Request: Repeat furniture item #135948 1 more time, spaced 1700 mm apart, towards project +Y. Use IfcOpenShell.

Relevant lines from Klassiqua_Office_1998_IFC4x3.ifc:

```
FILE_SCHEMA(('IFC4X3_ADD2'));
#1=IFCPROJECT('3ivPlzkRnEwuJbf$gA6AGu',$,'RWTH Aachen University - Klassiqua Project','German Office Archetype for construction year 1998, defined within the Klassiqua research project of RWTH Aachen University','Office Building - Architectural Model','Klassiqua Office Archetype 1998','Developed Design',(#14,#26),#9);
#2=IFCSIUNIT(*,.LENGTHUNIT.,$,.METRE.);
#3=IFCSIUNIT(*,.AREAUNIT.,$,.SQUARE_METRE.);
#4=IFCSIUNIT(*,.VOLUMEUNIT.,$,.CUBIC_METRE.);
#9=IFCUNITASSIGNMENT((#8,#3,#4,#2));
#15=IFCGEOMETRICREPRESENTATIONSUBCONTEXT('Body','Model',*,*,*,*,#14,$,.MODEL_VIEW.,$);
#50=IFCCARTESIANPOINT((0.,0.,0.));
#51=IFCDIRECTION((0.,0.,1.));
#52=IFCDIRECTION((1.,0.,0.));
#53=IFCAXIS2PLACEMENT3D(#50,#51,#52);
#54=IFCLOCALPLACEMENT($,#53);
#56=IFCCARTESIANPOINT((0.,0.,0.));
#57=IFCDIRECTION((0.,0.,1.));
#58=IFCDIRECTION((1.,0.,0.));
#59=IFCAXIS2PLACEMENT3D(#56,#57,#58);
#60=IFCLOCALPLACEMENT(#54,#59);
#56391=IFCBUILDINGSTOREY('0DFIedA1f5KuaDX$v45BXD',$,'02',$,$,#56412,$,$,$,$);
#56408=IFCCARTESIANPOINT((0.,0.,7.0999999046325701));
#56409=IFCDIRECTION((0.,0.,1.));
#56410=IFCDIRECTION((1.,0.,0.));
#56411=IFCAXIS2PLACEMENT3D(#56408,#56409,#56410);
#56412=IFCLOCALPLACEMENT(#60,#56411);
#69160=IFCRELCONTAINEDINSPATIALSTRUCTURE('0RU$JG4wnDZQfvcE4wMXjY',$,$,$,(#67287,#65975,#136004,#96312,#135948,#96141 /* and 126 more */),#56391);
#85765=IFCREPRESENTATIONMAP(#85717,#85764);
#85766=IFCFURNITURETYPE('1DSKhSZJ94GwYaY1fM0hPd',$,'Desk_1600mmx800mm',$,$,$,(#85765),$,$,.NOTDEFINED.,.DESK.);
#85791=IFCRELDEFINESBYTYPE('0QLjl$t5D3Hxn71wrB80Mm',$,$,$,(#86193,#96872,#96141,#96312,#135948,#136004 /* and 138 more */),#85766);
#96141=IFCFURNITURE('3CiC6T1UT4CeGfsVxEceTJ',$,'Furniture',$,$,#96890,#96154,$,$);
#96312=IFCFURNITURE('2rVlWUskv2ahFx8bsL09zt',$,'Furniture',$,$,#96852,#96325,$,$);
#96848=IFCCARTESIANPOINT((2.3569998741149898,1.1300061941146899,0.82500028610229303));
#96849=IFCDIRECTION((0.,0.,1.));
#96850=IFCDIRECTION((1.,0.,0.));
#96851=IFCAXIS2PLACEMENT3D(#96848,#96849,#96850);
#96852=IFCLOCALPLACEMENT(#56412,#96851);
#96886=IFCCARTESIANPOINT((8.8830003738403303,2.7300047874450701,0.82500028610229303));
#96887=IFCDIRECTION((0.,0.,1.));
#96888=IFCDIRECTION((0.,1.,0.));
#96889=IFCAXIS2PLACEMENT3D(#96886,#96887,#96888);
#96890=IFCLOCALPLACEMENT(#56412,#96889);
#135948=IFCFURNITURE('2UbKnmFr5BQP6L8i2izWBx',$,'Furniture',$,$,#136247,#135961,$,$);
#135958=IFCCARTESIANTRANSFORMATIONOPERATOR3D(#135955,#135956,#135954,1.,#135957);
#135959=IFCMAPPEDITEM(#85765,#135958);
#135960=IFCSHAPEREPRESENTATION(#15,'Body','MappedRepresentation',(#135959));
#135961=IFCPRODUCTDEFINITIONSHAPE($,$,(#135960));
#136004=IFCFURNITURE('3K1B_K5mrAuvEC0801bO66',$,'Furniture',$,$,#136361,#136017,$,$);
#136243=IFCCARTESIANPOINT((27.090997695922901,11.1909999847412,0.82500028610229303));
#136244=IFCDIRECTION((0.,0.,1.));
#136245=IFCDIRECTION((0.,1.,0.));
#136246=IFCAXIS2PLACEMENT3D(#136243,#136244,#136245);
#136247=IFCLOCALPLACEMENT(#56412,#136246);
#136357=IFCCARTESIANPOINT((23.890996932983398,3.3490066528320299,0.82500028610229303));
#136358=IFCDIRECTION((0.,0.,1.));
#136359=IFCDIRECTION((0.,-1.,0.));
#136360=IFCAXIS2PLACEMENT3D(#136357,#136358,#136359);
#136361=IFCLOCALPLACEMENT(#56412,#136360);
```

```python
import numpy as np
import ifcopenshell
import ifcopenshell.api.geometry
import ifcopenshell.api.root
import ifcopenshell.util.element
import ifcopenshell.util.placement

model = ifcopenshell.open("Klassiqua_Office_1998_IFC4x3.ifc")

source = model.by_guid("2UbKnmFr5BQP6L8i2izWBx")
base = ifcopenshell.util.placement.get_local_placement(source.ObjectPlacement)
step = np.array([0.0, 1.0, 0.0]) * 1.7

for i in range(1, 2):
    copy = ifcopenshell.api.root.copy_class(model, product=source)
    copy.Representation = ifcopenshell.util.element.copy_deep(
        model, source.Representation, exclude=["IfcGeometricRepresentationContext", "IfcRepresentationMap"]
    )
    matrix = base.copy()
    matrix[:3, 3] += i * step
    print("added at", matrix[:3, 3].round(3) + 0.0)
    ifcopenshell.api.geometry.edit_object_placement(model, product=copy, matrix=matrix, is_si=False)

model.write("Klassiqua_Office_1998_IFC4x3_updated.ifc")
```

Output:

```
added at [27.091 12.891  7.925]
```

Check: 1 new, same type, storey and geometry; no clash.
